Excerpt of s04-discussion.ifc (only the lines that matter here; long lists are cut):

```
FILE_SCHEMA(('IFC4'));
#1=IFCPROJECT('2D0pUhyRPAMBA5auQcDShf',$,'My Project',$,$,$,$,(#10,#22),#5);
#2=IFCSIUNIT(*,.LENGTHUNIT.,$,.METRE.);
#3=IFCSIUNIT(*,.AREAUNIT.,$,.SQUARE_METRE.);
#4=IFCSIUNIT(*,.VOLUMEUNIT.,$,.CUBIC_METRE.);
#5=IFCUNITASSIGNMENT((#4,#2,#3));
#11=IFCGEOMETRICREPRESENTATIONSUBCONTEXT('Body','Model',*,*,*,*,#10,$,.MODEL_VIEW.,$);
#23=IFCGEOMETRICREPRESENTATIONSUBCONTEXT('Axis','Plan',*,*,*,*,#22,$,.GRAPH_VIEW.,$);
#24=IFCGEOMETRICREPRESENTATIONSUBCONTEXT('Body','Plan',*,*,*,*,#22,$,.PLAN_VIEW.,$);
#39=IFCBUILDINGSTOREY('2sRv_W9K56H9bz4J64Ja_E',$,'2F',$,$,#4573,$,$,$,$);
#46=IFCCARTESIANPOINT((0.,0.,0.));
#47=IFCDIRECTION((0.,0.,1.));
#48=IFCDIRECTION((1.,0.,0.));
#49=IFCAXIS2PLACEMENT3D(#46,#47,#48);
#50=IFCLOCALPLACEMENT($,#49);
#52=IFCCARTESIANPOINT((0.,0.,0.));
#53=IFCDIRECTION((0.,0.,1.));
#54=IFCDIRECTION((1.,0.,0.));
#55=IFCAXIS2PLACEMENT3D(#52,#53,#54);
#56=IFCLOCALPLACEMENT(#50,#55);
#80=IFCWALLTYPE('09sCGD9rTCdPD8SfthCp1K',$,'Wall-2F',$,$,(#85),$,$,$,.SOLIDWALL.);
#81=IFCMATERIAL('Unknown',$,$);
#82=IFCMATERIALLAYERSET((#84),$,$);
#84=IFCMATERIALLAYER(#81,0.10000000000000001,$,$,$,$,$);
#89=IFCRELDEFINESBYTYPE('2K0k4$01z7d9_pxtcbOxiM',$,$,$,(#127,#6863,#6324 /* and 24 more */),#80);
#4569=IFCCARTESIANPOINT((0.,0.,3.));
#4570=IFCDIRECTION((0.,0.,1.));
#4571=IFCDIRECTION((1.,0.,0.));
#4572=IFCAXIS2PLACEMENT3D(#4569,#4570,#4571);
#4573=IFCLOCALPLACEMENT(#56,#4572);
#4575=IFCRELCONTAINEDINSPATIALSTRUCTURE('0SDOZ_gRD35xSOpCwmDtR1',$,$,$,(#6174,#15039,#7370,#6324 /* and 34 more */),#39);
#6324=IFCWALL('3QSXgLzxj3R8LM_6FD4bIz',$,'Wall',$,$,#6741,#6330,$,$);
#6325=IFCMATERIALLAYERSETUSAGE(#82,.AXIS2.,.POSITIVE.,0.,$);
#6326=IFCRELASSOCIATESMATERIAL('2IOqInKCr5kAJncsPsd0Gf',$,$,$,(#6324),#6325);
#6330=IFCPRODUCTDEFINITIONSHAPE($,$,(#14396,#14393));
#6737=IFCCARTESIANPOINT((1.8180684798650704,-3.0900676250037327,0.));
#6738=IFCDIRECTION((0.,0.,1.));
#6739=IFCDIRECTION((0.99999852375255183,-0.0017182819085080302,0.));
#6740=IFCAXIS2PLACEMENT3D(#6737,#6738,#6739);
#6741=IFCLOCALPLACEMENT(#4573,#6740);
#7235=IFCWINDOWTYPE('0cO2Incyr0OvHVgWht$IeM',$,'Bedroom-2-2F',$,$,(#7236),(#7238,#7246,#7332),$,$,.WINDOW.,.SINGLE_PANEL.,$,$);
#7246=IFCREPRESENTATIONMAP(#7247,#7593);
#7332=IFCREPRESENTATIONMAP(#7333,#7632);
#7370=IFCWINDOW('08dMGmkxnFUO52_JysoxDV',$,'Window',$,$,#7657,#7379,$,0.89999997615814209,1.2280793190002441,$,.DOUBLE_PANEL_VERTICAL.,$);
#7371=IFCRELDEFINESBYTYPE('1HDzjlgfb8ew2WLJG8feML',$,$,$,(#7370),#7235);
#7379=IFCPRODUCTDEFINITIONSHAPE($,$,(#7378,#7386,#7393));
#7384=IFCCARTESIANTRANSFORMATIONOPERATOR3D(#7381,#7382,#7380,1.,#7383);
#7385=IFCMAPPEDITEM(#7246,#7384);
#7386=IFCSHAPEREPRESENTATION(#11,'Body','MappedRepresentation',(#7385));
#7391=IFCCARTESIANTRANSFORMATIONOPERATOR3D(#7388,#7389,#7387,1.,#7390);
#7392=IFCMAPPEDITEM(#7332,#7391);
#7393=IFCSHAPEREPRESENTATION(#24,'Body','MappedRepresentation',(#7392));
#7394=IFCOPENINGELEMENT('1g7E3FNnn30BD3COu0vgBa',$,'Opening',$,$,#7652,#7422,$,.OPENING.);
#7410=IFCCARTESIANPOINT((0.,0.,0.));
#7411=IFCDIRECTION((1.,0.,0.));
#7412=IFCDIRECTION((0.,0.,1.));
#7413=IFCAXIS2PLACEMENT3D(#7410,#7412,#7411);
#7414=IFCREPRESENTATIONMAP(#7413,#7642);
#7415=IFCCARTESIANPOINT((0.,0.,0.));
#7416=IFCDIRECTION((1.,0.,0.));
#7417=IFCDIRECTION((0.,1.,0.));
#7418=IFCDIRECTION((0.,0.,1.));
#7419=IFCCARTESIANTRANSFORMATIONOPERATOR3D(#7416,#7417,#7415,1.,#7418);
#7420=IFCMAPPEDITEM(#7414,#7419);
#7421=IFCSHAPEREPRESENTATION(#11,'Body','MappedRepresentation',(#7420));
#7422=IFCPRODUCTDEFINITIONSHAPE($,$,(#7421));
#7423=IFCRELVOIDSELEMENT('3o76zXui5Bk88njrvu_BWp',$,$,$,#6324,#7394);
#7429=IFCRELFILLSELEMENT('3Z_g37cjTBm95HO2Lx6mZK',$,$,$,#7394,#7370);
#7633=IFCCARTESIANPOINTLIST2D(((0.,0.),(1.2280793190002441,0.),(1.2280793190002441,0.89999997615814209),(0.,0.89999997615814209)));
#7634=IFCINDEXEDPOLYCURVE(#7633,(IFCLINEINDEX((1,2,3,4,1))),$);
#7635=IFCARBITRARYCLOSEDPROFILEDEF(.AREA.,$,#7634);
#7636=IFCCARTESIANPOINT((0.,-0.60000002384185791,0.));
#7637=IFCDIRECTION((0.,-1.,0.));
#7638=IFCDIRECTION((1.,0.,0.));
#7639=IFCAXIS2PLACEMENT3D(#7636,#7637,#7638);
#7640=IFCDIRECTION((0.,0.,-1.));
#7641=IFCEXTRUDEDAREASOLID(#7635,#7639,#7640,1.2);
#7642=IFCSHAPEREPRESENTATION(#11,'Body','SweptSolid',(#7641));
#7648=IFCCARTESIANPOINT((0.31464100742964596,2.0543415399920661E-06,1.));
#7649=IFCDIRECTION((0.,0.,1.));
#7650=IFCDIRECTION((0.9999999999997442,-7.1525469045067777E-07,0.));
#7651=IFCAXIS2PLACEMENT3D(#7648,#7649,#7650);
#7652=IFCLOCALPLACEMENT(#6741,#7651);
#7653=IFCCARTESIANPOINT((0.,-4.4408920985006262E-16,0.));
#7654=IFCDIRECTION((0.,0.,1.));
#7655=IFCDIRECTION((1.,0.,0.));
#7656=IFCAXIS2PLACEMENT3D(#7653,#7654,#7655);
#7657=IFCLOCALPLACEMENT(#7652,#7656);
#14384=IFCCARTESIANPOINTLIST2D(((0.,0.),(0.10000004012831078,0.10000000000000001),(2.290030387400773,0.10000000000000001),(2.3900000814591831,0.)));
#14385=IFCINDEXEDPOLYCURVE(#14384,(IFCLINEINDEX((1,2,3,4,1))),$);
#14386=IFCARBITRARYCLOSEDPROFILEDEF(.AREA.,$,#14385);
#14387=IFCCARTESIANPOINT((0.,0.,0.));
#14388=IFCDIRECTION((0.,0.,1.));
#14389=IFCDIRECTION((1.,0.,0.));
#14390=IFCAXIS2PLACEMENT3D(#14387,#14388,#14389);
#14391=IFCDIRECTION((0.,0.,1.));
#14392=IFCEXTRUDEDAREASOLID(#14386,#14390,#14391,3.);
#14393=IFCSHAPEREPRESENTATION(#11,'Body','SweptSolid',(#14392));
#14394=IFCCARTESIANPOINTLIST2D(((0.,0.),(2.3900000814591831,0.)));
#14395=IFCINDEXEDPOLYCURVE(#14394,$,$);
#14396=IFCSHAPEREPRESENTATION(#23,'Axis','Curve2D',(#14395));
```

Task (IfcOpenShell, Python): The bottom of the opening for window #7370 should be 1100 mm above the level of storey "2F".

```python
import numpy as np
import ifcopenshell
import ifcopenshell.api.geometry
import ifcopenshell.geom
import ifcopenshell.util.element
import ifcopenshell.util.placement
import ifcopenshell.util.shape
import ifcopenshell.util.unit

model = ifcopenshell.open("s04-discussion.ifc")
unit_scale = ifcopenshell.util.unit.calculate_unit_scale(model)

window = model.by_guid("08dMGmkxnFUO52_JysoxDV")
opening = window.FillsVoids[0].RelatingOpeningElement
storey = ifcopenshell.util.element.get_container(window, ifc_class="IfcBuildingStorey")
level = ifcopenshell.util.placement.get_local_placement(storey.ObjectPlacement)[2, 3]

# The opening's origin need not be at the sill, so measure its lowest point.
shape = ifcopenshell.geom.create_shape(ifcopenshell.geom.settings(), opening)
bottom = ifcopenshell.util.shape.get_shape_bottom_elevation(shape, shape.geometry) / unit_scale
dz = level + 1.1 - bottom

shift = np.array([0.0, 0.0, dz])
# The window is placed relative to its opening, so it follows when the opening moves.
matrix = ifcopenshell.util.placement.get_local_placement(opening.ObjectPlacement)
matrix[:3, 3] += shift
ifcopenshell.api.geometry.edit_object_placement(
    model, product=opening, matrix=matrix, is_si=False, should_transform_children=True
)

print(f"moved by {dz * unit_scale:+.3f} m")

model.write("s04-discussion_v2.ifc")
```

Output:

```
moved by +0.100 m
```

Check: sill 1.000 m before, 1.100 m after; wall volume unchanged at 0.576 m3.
